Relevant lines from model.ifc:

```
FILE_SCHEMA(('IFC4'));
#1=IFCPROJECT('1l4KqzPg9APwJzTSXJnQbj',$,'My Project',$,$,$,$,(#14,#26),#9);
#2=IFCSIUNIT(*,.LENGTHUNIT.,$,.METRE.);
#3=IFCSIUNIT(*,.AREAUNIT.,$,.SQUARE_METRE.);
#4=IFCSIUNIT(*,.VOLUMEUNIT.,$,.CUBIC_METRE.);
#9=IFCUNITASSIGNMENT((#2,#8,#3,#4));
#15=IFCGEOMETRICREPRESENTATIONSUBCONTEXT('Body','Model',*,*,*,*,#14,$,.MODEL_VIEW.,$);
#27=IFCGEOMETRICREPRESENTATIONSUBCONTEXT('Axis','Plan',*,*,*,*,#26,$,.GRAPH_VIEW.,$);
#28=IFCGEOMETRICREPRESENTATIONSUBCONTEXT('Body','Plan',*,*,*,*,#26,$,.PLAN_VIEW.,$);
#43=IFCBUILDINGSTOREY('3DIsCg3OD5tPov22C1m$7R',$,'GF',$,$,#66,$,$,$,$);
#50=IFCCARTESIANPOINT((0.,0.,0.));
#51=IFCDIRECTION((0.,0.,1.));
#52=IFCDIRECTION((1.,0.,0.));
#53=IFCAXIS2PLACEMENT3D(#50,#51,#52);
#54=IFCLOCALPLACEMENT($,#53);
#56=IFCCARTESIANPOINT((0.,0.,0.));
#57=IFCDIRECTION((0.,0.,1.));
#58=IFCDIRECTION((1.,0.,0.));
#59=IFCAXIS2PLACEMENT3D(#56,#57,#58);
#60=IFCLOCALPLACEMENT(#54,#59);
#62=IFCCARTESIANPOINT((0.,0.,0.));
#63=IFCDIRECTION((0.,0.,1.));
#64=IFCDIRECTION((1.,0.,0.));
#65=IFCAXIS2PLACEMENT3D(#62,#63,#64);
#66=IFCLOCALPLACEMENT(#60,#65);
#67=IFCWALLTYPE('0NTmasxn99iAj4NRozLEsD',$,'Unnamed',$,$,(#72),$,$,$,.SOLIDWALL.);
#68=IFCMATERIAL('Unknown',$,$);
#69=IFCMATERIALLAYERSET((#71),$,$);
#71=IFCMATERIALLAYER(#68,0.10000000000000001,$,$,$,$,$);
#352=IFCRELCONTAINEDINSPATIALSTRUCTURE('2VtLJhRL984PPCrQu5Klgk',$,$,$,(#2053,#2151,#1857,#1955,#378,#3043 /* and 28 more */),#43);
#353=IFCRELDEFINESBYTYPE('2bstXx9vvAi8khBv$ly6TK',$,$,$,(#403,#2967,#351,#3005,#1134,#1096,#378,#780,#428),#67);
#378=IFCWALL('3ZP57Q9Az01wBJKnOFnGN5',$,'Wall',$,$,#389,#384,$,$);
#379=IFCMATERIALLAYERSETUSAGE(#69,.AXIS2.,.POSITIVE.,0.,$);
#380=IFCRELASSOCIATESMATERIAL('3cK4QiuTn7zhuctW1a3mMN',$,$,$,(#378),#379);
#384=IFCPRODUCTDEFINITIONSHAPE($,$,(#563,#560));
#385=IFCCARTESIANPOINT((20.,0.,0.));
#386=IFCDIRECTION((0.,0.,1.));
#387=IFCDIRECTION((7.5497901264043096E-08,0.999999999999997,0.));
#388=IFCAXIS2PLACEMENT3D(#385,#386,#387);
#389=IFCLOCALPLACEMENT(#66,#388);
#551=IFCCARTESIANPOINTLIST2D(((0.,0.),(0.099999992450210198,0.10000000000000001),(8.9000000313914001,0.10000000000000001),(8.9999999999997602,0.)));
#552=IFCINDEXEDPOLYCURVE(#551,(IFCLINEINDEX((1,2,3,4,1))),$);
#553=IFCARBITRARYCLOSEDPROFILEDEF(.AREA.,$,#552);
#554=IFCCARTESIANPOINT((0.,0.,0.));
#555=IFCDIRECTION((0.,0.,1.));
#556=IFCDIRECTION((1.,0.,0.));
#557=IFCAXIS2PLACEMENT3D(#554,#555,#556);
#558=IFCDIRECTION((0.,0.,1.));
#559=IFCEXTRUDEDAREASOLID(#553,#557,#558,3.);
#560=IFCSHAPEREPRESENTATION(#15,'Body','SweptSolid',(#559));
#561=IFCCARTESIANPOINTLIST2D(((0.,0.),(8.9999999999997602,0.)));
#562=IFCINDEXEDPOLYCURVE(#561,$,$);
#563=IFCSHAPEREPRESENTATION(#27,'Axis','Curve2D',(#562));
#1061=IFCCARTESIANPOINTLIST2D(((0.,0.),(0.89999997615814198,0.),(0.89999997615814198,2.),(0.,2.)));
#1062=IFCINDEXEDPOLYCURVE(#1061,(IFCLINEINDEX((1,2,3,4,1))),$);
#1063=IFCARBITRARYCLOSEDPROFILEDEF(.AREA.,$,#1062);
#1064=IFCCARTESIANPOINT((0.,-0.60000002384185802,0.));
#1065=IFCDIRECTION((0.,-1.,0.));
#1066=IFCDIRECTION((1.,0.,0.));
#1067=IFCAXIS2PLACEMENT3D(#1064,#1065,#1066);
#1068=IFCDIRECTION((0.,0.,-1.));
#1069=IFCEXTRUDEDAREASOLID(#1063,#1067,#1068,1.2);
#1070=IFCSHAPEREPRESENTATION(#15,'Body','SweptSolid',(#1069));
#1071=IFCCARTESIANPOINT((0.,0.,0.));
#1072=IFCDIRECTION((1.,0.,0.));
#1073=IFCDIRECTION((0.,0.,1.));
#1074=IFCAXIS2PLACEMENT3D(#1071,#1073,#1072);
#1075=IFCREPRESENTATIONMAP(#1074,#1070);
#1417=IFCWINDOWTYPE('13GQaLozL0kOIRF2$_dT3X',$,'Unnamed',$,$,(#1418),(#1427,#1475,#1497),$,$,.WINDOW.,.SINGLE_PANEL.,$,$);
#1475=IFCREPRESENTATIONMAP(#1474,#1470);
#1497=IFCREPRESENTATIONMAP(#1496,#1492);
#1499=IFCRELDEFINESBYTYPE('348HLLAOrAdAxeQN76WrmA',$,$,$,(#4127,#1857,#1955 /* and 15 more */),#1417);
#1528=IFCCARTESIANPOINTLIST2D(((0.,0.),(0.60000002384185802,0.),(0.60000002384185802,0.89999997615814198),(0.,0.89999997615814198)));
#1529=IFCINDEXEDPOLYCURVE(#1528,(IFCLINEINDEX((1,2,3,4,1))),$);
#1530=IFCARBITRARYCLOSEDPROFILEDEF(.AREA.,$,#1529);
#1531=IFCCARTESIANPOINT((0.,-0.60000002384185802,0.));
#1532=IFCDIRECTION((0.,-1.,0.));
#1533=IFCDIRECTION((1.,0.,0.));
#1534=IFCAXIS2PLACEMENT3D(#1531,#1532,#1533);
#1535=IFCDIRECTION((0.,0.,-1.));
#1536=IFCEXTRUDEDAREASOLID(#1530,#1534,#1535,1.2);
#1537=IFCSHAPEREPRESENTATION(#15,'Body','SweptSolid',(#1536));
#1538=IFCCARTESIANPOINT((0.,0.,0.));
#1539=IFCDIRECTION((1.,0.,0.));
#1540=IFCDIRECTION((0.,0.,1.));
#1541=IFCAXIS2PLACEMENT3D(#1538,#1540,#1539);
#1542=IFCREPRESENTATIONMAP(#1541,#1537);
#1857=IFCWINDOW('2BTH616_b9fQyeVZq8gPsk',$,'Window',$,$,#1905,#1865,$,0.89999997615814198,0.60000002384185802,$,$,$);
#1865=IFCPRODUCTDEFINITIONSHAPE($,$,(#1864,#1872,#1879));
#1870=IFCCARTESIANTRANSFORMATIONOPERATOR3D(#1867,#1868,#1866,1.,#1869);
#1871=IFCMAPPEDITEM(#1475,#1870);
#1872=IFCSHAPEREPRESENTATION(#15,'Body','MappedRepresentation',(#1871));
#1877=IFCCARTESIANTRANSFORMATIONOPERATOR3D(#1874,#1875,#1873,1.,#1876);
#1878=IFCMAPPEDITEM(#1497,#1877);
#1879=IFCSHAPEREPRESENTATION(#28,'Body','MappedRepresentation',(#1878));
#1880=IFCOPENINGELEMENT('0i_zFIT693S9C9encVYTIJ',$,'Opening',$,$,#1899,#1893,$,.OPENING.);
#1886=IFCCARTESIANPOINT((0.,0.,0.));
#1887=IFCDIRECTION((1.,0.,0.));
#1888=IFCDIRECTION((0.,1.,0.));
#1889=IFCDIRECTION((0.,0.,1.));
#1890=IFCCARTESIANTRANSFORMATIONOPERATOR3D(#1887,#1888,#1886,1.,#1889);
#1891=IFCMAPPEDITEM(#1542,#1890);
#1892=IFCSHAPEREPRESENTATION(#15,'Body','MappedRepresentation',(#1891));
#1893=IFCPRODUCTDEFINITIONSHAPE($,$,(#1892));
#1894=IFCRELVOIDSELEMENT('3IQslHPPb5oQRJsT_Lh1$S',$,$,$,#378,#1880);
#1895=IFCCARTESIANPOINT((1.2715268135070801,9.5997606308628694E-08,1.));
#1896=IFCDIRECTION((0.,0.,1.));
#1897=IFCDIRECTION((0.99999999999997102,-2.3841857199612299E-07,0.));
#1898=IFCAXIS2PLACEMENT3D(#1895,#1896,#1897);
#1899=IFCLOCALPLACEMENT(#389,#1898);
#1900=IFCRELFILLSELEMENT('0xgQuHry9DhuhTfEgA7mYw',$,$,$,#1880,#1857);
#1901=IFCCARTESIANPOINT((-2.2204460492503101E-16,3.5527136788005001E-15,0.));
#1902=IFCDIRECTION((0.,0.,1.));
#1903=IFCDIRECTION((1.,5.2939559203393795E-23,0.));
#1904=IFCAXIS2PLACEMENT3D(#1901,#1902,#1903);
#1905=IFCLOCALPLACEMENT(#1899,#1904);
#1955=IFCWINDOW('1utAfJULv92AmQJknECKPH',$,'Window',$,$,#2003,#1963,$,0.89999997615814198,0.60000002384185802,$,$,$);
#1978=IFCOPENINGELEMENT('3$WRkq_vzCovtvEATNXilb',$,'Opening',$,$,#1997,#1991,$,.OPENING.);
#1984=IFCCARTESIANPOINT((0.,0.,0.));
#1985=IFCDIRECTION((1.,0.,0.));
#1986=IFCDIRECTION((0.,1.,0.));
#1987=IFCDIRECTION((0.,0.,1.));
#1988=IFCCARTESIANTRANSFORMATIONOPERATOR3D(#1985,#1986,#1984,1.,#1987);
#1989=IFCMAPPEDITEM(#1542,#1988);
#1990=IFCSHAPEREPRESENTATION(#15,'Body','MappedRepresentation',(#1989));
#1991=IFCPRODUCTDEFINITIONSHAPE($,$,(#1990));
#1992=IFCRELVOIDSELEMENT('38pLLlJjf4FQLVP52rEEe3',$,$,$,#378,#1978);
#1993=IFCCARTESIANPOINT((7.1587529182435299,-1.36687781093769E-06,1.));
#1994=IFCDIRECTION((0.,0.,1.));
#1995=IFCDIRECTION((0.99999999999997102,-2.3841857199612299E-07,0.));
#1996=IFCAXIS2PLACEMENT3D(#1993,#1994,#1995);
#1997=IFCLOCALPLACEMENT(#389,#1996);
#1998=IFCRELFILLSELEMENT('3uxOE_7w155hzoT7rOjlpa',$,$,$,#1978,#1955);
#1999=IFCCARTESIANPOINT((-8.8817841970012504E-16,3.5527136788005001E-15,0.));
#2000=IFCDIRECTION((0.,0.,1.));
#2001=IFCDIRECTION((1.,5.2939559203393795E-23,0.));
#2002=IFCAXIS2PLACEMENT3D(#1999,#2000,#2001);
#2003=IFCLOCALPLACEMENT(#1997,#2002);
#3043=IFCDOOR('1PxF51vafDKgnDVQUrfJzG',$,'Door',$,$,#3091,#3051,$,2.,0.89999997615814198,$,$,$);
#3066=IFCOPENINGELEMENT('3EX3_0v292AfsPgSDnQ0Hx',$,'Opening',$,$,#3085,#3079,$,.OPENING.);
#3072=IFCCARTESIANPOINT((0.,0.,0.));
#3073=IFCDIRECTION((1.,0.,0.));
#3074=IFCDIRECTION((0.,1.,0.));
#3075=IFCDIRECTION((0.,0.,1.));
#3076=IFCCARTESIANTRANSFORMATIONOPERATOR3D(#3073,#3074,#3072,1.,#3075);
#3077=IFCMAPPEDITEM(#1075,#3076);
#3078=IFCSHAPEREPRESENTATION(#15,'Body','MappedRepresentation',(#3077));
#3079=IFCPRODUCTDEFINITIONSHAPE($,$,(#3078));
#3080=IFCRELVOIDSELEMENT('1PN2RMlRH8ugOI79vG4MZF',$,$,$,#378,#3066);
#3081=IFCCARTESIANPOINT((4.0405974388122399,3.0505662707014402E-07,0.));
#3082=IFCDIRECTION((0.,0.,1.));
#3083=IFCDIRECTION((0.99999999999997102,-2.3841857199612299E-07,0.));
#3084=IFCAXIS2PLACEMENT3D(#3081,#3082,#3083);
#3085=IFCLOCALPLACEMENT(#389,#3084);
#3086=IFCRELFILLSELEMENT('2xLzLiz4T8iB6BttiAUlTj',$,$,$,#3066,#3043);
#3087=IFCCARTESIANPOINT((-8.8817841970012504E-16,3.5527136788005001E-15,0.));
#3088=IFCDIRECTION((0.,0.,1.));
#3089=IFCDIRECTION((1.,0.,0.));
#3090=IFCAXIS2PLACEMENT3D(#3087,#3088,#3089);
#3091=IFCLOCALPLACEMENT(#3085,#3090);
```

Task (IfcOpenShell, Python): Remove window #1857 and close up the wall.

```python
import ifcopenshell
import ifcopenshell.api.feature
import ifcopenshell.api.root
import ifcopenshell.geom
import ifcopenshell.util.shape

model = ifcopenshell.open("model.ifc")
settings = ifcopenshell.geom.settings()


def volume(element):
    """Net volume in cubic metres, openings subtracted."""
    shape = ifcopenshell.geom.create_shape(settings, element)
    return ifcopenshell.util.shape.get_volume(shape.geometry)


window = model.by_id(1857)
opening = window.FillsVoids[0].RelatingOpeningElement
wall = opening.VoidsElements[0].RelatingBuildingElement
before = volume(wall)

ifcopenshell.api.root.remove_product(model, product=window)
ifcopenshell.api.feature.remove_feature(model, feature=opening)

after = volume(wall)

print(f"wall volume {before:.3f} -> {after:.3f} m3")

model.write("model_edited.ifc")
```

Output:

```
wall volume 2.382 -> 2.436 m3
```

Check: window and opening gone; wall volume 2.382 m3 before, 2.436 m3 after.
